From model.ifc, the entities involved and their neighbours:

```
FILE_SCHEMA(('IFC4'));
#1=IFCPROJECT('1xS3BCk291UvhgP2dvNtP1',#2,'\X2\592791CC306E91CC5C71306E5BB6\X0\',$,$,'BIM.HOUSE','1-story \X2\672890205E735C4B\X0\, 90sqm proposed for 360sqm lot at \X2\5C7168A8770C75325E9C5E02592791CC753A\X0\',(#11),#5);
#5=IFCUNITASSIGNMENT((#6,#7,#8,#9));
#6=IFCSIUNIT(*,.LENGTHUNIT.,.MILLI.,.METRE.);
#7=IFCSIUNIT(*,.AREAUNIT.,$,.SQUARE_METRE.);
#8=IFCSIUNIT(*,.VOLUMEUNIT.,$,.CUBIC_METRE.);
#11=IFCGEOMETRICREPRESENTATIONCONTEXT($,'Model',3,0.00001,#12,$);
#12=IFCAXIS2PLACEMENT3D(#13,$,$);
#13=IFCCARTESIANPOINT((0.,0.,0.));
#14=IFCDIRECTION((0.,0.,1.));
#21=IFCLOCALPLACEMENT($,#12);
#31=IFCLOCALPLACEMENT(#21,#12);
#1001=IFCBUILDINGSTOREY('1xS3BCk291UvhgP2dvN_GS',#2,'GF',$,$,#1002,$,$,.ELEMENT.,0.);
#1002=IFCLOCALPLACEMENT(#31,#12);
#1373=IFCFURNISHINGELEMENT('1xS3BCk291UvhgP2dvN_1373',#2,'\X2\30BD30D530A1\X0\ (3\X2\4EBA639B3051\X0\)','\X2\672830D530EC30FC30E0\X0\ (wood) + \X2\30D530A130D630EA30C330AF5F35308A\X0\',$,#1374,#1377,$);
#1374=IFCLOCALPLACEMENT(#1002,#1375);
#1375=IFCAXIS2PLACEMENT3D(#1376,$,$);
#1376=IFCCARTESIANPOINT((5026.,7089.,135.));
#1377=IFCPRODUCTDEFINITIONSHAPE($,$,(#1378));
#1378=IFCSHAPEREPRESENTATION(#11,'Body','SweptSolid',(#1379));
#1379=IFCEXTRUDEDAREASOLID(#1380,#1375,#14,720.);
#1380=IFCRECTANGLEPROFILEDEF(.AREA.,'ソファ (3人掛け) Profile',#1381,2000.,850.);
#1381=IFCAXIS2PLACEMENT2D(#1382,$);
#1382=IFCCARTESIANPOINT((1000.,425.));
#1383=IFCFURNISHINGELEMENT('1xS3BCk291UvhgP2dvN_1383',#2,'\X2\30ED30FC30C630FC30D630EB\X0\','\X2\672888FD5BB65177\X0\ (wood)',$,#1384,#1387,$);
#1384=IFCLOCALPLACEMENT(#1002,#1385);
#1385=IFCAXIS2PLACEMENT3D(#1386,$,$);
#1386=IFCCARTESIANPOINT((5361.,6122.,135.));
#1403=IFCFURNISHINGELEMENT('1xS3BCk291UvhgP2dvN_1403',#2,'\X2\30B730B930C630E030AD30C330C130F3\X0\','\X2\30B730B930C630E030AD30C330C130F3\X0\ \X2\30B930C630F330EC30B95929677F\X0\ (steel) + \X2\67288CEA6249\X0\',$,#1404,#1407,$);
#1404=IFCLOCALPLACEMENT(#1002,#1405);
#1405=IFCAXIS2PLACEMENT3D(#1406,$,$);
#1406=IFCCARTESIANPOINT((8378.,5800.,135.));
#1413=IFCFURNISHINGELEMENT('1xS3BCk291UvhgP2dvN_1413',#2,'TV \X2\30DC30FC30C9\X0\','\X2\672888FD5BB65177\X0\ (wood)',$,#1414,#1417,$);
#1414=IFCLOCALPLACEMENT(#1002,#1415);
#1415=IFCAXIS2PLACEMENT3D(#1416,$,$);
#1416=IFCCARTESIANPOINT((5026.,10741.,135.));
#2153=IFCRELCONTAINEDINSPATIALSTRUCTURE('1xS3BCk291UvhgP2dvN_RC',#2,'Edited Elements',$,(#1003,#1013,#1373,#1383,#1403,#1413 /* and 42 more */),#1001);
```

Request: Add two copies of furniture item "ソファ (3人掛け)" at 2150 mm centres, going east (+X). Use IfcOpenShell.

```python
import numpy as np
import ifcopenshell
import ifcopenshell.api.geometry
import ifcopenshell.api.root
import ifcopenshell.util.element
import ifcopenshell.util.placement

model = ifcopenshell.open("model.ifc")


def reuse_history(source, copy):
    """copy_class also copies each property set's owner history, people and application; keep the originals."""
    for rel in copy.IsDefinedBy:
        if rel.is_a("IfcRelDefinesByProperties") and (history := rel.RelatingPropertyDefinition.OwnerHistory):
            rel.RelatingPropertyDefinition.OwnerHistory = source.OwnerHistory
            ifcopenshell.util.element.remove_deep2(model, history)


source = model.by_guid("1xS3BCk291UvhgP2dvN_1373")
base = ifcopenshell.util.placement.get_local_placement(source.ObjectPlacement)
step = np.array([1.0, 0.0, 0.0]) * 2150.0

for i in range(1, 3):
    copy = ifcopenshell.api.root.copy_class(model, product=source)
    copy.Representation = ifcopenshell.util.element.copy_deep(
        model, source.Representation, exclude=["IfcGeometricRepresentationContext", "IfcRepresentationMap"]
    )
    reuse_history(source, copy)
    matrix = base.copy()
    matrix[:3, 3] += i * step
    print("added at", matrix[:3, 3].round(3) + 0.0)
    ifcopenshell.api.geometry.edit_object_placement(model, product=copy, matrix=matrix, is_si=False)

model.write("model_rev.ifc")
```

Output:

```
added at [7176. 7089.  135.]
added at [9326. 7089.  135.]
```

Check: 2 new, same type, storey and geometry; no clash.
